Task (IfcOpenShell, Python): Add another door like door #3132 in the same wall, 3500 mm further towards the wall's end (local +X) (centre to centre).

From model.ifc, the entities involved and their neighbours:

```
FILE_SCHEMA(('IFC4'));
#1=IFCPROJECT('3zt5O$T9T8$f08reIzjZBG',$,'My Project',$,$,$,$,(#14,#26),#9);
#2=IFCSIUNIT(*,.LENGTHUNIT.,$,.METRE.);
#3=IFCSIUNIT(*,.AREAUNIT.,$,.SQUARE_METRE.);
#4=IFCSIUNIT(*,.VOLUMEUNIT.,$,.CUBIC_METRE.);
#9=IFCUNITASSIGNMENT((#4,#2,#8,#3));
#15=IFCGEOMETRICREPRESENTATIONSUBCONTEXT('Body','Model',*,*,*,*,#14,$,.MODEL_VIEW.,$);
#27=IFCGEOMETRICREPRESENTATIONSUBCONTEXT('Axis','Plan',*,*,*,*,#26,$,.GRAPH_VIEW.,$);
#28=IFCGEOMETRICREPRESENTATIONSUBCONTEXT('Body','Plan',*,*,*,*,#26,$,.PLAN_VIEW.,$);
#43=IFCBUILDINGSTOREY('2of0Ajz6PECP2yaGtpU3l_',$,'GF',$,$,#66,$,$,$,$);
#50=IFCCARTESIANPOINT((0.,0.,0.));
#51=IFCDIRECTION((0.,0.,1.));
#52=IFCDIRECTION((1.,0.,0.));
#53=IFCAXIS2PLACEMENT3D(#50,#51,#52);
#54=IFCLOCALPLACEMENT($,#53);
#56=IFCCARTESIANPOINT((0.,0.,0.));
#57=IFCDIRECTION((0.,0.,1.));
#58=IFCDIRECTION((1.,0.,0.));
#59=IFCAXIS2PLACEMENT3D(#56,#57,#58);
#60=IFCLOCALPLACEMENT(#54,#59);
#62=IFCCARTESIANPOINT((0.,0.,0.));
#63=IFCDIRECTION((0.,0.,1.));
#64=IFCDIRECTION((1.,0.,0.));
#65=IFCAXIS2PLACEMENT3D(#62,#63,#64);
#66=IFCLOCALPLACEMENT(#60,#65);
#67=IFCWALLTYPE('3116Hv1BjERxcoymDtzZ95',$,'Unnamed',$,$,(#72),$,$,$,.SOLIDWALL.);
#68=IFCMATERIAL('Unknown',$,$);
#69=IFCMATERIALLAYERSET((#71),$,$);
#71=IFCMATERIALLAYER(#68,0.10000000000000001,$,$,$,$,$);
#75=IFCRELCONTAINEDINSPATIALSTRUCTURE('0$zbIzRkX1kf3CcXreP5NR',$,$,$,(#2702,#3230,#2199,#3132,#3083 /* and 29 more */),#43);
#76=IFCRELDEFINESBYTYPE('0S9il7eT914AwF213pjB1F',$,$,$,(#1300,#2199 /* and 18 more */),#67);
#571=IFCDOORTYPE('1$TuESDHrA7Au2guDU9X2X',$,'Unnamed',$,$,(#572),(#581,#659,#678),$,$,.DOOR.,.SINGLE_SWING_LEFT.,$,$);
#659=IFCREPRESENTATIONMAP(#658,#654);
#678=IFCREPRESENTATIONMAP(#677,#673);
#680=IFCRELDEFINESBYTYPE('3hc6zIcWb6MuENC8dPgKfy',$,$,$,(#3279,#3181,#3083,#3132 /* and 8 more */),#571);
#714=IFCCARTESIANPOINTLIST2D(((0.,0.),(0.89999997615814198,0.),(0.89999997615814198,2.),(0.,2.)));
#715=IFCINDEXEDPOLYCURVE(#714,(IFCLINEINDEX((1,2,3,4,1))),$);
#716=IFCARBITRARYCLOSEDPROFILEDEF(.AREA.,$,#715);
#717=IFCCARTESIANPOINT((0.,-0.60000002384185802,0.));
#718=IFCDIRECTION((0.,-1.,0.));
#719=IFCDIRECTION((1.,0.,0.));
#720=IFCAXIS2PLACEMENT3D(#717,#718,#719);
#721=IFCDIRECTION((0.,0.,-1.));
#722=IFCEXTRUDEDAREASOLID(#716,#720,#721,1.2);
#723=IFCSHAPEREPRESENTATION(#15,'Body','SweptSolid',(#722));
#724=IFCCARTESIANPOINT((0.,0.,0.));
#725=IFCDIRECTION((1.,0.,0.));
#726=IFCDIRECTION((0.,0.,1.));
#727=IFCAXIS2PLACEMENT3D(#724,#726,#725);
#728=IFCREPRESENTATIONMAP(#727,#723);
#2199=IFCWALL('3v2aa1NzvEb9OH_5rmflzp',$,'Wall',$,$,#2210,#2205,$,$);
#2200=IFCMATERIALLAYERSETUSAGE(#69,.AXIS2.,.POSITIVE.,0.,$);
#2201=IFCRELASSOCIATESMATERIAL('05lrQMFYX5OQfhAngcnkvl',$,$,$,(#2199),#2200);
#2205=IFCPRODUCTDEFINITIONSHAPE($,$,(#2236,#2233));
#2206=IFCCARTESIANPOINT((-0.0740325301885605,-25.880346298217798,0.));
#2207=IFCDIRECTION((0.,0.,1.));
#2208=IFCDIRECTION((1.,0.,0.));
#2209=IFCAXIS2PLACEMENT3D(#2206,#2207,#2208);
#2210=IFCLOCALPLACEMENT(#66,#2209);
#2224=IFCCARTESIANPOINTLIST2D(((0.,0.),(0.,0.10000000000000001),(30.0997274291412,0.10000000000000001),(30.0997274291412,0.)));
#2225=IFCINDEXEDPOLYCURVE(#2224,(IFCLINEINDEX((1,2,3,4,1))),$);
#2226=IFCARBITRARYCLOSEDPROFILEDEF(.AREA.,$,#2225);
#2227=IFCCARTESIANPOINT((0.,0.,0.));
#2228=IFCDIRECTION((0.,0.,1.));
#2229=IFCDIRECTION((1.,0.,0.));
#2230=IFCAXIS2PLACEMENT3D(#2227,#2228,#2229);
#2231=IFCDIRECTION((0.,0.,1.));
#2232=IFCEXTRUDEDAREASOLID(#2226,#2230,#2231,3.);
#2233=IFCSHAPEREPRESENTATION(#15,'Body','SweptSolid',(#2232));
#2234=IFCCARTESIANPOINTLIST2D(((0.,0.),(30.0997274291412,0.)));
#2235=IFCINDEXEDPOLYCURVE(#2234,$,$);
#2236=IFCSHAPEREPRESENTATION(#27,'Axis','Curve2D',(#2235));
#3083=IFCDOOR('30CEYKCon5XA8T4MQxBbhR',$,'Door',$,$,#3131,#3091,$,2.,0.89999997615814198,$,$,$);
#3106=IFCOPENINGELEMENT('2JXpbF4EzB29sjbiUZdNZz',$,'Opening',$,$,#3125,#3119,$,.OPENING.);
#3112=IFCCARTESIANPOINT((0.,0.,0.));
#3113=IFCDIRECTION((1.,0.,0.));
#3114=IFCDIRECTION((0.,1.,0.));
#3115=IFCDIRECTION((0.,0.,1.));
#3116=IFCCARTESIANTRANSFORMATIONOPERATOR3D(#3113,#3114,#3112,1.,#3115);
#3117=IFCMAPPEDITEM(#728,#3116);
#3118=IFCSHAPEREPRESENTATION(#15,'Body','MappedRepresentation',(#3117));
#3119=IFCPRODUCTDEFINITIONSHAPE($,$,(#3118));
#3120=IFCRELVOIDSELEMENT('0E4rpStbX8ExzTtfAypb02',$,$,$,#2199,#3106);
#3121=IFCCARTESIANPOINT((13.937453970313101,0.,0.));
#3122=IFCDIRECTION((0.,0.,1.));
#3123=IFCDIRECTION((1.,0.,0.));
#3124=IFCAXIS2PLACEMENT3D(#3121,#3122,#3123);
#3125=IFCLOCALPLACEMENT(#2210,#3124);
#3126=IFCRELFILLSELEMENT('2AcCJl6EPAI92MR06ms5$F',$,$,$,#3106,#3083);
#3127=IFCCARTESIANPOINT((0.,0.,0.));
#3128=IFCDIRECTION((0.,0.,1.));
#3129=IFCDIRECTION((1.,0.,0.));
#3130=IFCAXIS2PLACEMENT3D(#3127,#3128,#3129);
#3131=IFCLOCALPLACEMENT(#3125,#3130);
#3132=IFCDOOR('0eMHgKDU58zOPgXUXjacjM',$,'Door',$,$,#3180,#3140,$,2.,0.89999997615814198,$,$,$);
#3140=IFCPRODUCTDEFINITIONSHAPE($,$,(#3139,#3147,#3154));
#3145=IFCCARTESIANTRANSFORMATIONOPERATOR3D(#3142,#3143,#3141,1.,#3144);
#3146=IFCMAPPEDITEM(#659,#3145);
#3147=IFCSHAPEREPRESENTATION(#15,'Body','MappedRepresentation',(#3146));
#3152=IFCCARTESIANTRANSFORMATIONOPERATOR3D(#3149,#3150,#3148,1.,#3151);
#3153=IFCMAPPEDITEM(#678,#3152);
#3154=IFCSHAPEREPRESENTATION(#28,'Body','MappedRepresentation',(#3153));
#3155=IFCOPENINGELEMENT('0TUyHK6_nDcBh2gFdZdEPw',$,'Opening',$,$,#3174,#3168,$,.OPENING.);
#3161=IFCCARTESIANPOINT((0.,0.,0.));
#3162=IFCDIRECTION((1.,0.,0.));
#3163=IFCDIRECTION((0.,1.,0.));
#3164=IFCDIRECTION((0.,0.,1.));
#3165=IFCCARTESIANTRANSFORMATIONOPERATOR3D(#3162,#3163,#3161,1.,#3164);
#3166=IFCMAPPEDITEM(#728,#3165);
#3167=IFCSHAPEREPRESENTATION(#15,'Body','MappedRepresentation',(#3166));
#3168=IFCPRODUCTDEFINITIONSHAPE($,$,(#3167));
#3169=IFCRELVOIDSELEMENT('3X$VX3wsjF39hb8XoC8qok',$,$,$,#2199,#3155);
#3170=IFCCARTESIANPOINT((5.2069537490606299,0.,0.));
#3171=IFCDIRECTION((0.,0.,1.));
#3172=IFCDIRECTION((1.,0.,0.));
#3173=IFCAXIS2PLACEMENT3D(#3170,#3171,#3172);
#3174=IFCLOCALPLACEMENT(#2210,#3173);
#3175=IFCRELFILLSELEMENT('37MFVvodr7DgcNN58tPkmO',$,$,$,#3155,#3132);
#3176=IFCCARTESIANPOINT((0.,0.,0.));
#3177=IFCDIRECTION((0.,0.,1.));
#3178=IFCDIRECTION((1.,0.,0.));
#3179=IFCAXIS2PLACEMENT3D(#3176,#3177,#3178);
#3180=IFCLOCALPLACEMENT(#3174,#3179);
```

```python
import ifcopenshell
import ifcopenshell.api.feature
import ifcopenshell.api.geometry
import ifcopenshell.api.root
import ifcopenshell.geom
import ifcopenshell.util.element
import ifcopenshell.util.placement
import ifcopenshell.util.shape

model = ifcopenshell.open("model.ifc")
settings = ifcopenshell.geom.settings()


def volume(element):
    """Net volume in cubic metres, openings subtracted."""
    shape = ifcopenshell.geom.create_shape(settings, element)
    return ifcopenshell.util.shape.get_volume(shape.geometry)


door = model.by_guid("0eMHgKDU58zOPgXUXjacjM")
opening = door.FillsVoids[0].RelatingOpeningElement
wall = opening.VoidsElements[0].RelatingBuildingElement
before = volume(wall)
shift = ifcopenshell.util.placement.get_local_placement(wall.ObjectPlacement)[:3, 0] * 3.5

# copy_class copies the void relationship, type, container and properties, but no geometry.
new_opening = ifcopenshell.api.root.copy_class(model, product=opening)
new_opening.Representation = ifcopenshell.util.element.copy_deep(
    model, opening.Representation, exclude=["IfcGeometricRepresentationContext", "IfcRepresentationMap"]
)
new_door = ifcopenshell.api.root.copy_class(model, product=door)
new_door.Representation = ifcopenshell.util.element.copy_deep(
    model, door.Representation, exclude=["IfcGeometricRepresentationContext", "IfcRepresentationMap"]
)
ifcopenshell.api.feature.add_filling(model, opening=new_opening, element=new_door)

for old, new in ((opening, new_opening), (door, new_door)):
    matrix = ifcopenshell.util.placement.get_local_placement(old.ObjectPlacement)
    matrix[:3, 3] += shift
    ifcopenshell.api.geometry.edit_object_placement(model, product=new, matrix=matrix, is_si=False)

after = volume(wall)

print(f"wall volume {before:.3f} -> {after:.3f} m3")

model.write("model-out.ifc")
```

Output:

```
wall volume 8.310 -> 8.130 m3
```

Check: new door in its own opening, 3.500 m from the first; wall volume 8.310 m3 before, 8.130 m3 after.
